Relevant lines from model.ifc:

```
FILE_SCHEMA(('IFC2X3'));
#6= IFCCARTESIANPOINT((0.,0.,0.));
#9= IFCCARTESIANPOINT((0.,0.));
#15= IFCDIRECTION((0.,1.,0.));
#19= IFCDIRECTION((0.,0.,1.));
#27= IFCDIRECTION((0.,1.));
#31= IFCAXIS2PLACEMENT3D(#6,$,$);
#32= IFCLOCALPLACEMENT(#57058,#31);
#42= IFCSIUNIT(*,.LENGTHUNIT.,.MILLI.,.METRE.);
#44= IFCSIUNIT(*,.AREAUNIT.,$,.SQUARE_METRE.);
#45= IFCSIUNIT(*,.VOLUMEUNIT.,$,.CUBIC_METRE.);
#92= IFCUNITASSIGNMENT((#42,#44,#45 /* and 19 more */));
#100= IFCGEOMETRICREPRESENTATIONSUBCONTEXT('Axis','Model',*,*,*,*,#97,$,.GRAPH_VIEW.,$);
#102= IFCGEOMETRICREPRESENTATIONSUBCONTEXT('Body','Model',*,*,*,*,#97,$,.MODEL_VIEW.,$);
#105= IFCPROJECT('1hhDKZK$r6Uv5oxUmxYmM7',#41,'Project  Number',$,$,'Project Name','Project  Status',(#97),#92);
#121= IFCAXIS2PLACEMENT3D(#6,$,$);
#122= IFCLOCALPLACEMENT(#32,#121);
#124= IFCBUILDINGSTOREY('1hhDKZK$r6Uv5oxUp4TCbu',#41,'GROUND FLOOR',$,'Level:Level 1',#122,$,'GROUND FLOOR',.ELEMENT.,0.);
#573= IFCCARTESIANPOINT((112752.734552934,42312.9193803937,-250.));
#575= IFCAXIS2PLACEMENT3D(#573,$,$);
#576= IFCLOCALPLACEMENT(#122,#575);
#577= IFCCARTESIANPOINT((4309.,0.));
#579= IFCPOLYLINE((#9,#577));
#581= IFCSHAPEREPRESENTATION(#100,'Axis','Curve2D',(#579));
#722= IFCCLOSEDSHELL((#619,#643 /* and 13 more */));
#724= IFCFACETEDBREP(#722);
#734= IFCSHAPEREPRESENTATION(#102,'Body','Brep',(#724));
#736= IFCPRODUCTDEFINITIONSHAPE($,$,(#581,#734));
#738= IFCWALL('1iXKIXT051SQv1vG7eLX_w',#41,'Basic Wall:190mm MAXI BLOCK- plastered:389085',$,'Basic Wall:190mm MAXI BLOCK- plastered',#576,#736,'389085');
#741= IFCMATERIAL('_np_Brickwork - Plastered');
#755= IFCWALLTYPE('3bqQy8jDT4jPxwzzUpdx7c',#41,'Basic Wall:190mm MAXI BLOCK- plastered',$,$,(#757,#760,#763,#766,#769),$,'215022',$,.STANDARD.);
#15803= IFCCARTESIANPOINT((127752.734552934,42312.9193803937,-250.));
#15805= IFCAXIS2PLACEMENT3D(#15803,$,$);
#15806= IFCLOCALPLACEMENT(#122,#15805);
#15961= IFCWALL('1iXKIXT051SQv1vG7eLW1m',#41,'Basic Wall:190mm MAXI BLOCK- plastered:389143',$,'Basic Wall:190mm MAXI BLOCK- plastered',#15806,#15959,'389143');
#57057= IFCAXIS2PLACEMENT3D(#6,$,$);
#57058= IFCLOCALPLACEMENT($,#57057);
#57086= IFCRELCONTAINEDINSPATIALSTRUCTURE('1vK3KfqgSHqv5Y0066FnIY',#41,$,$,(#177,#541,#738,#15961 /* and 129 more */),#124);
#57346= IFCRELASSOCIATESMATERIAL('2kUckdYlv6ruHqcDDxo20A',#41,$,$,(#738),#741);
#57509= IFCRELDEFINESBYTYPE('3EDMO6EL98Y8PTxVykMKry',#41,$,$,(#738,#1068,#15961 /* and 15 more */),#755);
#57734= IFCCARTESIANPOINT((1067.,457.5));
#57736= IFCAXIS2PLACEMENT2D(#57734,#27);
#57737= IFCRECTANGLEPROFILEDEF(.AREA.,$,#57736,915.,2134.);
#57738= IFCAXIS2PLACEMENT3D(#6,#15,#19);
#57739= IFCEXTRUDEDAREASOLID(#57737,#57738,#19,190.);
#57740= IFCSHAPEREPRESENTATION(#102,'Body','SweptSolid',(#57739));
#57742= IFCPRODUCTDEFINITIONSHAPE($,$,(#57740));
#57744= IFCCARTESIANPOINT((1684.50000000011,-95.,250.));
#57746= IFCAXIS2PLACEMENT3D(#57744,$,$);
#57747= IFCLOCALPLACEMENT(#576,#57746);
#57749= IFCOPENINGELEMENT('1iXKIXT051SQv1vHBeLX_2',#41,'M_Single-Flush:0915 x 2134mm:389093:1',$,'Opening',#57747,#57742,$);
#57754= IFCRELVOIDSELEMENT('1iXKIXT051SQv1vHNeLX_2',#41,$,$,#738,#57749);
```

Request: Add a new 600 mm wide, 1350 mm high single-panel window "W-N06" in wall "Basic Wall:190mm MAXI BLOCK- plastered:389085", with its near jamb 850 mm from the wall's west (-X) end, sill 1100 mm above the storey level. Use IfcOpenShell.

```python
import numpy as np
import ifcopenshell
import ifcopenshell.api.feature
import ifcopenshell.api.geometry
import ifcopenshell.api.root
import ifcopenshell.api.spatial
import ifcopenshell.api.type
import ifcopenshell.geom
import ifcopenshell.util.element
import ifcopenshell.util.placement
import ifcopenshell.util.representation
import ifcopenshell.util.shape
import ifcopenshell.util.unit

model = ifcopenshell.open("model.ifc")
unit_scale = ifcopenshell.util.unit.calculate_unit_scale(model)
settings = ifcopenshell.geom.settings()


def volume(element):
    """Net volume in cubic metres, openings subtracted."""
    shape = ifcopenshell.geom.create_shape(settings, element)
    return ifcopenshell.util.shape.get_volume(shape.geometry)


wall = model.by_guid("1iXKIXT051SQv1vG7eLX_w")
storey = ifcopenshell.util.element.get_container(wall, ifc_class="IfcBuildingStorey")
context = ifcopenshell.util.representation.get_context(model, "Model", "Body", "MODEL_VIEW")
before = volume(wall)

width, height, from_end, sill = 0.6, 1.35, 0.85, 1.1  # metres

# The wall runs along its own X axis, and the end named is its -X end.
wall_shape = ifcopenshell.geom.create_shape(settings, wall)
x, y, z = ifcopenshell.util.shape.get_vertices(wall_shape.geometry).T
start = x.min() + from_end
face, thickness = float(y.min()), float(y.max() - y.min())
wall_matrix = ifcopenshell.util.placement.get_local_placement(wall.ObjectPlacement)
level = ifcopenshell.util.placement.get_local_placement(storey.ObjectPlacement)[2, 3]


def in_wall(x, y):
    """Placement at x, y metres in the wall's axes, at sill height."""
    matrix = wall_matrix.copy()
    matrix[:, 3] = wall_matrix @ np.array([x / unit_scale, y / unit_scale, 0.0, 1.0])
    matrix[2, 3] = level + sill / unit_scale
    return matrix


# Opening: a box that overshoots both wall faces by 50 mm.
opening = ifcopenshell.api.root.create_entity(model, ifc_class="IfcOpeningElement")
box = ifcopenshell.api.geometry.add_wall_representation(
    model, context=context, length=width, height=height, thickness=thickness + 0.1
)
ifcopenshell.api.geometry.assign_representation(model, product=opening, representation=box)
ifcopenshell.api.geometry.edit_object_placement(model, product=opening, matrix=in_wall(start, face - 0.05), is_si=False)
ifcopenshell.api.feature.add_feature(model, feature=opening, element=wall)

window = ifcopenshell.api.root.create_entity(model, ifc_class="IfcWindow", name="W-N06")
window.OverallWidth, window.OverallHeight = width / unit_scale, height / unit_scale
body = ifcopenshell.api.geometry.add_window_representation(
    model,
    context=context,
    overall_width=window.OverallWidth,
    overall_height=window.OverallHeight,
    partition_type="SINGLE_PANEL",
)
ifcopenshell.api.geometry.assign_representation(model, product=window, representation=body)
ifcopenshell.api.spatial.assign_container(model, products=[window], relating_structure=storey)
fills = ifcopenshell.api.feature.add_filling(model, opening=opening, element=window)
fills.OwnerHistory = window.OwnerHistory  # required in IFC2X3

# IFC2X3 keeps the operation on the window style.
style = ifcopenshell.api.root.create_entity(model, ifc_class="IfcWindowStyle", name="W-N06")
style.OperationType, style.ConstructionType = "SINGLE_PANEL", "NOTDEFINED"
style.ParameterTakesPrecedence = style.Sizeable = False
ifcopenshell.api.type.assign_type(model, related_objects=[window], relating_type=style)

# Centre the window in the wall's thickness.
ifcopenshell.api.geometry.edit_object_placement(model, product=window, matrix=in_wall(start, face), is_si=False)
window_shape = ifcopenshell.geom.create_shape(settings, window)
depth = ifcopenshell.util.shape.get_vertices(window_shape.geometry)[:, 1]
offset = face + thickness / 2 - (depth.min() + depth.max()) / 2
ifcopenshell.api.geometry.edit_object_placement(model, product=window, matrix=in_wall(start, offset), is_si=False)

after = volume(wall)

print(f"wall volume {before:.3f} -> {after:.3f} m3")

model.write("model_updated.ifc")
```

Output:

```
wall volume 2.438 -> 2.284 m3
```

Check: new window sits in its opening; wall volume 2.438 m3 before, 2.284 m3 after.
